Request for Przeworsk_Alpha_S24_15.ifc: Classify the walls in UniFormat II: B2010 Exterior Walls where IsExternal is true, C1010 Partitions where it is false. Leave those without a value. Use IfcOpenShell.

First a look at what the model holds.

```python
import ifcopenshell
import ifcopenshell.util.element

model = ifcopenshell.open("Przeworsk_Alpha_S24_15.ifc")
print(model.schema)
print("classifications:", [c.Name for c in model.by_type("IfcClassification")])
values = [ifcopenshell.util.element.get_pset(e, "Pset_WallCommon", "IsExternal") for e in model.by_type("IfcWall")]
for value in (True, False, None):
    print("IsExternal", value, values.count(value))
```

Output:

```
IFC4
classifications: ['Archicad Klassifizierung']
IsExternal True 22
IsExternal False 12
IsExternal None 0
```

```python
import ifcopenshell
import ifcopenshell.api.classification
import ifcopenshell.util.element

model = ifcopenshell.open("Przeworsk_Alpha_S24_15.ifc")

system = ifcopenshell.api.classification.add_classification(model, classification="UniFormat II")

walls = model.by_type("IfcWall")
external = {e: ifcopenshell.util.element.get_pset(e, "Pset_WallCommon", "IsExternal") for e in walls}
for flag, code, name in ((True, "B2010", "Exterior Walls"), (False, "C1010", "Partitions")):
    products = [e for e in walls if external[e] is flag]
    ifcopenshell.api.classification.add_reference(
        model, products=products, classification=system, identification=code, name=name
    )
    print(code, len(products))

model.write("Przeworsk_Alpha_S24_15-out.ifc")
```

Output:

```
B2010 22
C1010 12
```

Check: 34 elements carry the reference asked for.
